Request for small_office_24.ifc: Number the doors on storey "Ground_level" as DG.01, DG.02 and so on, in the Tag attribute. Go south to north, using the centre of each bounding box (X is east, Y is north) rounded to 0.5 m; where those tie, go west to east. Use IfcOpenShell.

First a look at what the model holds.

```python
import ifcopenshell
import ifcopenshell.util.element
import ifcopenshell.util.placement

model = ifcopenshell.open("small_office_24.ifc")
print(model.schema)
storey = next(s for s in model.by_type("IfcBuildingStorey") if s.Name == "Ground_level")
doors = [e for e in ifcopenshell.util.element.get_decomposition(storey) if e.is_a("IfcDoor")]
for e in sorted(doors, key=lambda e: e.id()):
    origin = ifcopenshell.util.placement.get_local_placement(e.ObjectPlacement)[:3, 3]
    print(e.id(), e.Tag, e.Name, origin.round(2) + 0.0, sep=" | ")
```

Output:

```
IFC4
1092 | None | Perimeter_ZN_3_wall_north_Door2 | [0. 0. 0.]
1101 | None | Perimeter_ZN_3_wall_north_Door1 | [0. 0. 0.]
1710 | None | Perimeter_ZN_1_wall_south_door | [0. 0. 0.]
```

```python
import ifcopenshell
import ifcopenshell.geom
import ifcopenshell.util.element
import ifcopenshell.util.shape

model = ifcopenshell.open("small_office_24.ifc")
settings = ifcopenshell.geom.settings()
settings.set("use-world-coords", True)


def centre(element):
    shape = ifcopenshell.geom.create_shape(settings, element)
    return ifcopenshell.util.shape.get_bbox_centroid(shape.geometry)


storey = next(s for s in model.by_type("IfcBuildingStorey") if s.Name == "Ground_level")
doors = [e for e in ifcopenshell.util.element.get_decomposition(storey) if e.is_a("IfcDoor")]

# Insertion points can sit at a corner or the storey origin, so sort by the geometry (in metres).
centres = {e: centre(e) for e in doors}
doors.sort(key=lambda e: (round(centres[e][1] / 0.5), centres[e][0]))

for i, e in enumerate(doors, start=1):
    number = f"DG.{i:02d}"
    e.Tag = number
    print(e.id(), number)

model.write("small_office_24_v2.ifc")
```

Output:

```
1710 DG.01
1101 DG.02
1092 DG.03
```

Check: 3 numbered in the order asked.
